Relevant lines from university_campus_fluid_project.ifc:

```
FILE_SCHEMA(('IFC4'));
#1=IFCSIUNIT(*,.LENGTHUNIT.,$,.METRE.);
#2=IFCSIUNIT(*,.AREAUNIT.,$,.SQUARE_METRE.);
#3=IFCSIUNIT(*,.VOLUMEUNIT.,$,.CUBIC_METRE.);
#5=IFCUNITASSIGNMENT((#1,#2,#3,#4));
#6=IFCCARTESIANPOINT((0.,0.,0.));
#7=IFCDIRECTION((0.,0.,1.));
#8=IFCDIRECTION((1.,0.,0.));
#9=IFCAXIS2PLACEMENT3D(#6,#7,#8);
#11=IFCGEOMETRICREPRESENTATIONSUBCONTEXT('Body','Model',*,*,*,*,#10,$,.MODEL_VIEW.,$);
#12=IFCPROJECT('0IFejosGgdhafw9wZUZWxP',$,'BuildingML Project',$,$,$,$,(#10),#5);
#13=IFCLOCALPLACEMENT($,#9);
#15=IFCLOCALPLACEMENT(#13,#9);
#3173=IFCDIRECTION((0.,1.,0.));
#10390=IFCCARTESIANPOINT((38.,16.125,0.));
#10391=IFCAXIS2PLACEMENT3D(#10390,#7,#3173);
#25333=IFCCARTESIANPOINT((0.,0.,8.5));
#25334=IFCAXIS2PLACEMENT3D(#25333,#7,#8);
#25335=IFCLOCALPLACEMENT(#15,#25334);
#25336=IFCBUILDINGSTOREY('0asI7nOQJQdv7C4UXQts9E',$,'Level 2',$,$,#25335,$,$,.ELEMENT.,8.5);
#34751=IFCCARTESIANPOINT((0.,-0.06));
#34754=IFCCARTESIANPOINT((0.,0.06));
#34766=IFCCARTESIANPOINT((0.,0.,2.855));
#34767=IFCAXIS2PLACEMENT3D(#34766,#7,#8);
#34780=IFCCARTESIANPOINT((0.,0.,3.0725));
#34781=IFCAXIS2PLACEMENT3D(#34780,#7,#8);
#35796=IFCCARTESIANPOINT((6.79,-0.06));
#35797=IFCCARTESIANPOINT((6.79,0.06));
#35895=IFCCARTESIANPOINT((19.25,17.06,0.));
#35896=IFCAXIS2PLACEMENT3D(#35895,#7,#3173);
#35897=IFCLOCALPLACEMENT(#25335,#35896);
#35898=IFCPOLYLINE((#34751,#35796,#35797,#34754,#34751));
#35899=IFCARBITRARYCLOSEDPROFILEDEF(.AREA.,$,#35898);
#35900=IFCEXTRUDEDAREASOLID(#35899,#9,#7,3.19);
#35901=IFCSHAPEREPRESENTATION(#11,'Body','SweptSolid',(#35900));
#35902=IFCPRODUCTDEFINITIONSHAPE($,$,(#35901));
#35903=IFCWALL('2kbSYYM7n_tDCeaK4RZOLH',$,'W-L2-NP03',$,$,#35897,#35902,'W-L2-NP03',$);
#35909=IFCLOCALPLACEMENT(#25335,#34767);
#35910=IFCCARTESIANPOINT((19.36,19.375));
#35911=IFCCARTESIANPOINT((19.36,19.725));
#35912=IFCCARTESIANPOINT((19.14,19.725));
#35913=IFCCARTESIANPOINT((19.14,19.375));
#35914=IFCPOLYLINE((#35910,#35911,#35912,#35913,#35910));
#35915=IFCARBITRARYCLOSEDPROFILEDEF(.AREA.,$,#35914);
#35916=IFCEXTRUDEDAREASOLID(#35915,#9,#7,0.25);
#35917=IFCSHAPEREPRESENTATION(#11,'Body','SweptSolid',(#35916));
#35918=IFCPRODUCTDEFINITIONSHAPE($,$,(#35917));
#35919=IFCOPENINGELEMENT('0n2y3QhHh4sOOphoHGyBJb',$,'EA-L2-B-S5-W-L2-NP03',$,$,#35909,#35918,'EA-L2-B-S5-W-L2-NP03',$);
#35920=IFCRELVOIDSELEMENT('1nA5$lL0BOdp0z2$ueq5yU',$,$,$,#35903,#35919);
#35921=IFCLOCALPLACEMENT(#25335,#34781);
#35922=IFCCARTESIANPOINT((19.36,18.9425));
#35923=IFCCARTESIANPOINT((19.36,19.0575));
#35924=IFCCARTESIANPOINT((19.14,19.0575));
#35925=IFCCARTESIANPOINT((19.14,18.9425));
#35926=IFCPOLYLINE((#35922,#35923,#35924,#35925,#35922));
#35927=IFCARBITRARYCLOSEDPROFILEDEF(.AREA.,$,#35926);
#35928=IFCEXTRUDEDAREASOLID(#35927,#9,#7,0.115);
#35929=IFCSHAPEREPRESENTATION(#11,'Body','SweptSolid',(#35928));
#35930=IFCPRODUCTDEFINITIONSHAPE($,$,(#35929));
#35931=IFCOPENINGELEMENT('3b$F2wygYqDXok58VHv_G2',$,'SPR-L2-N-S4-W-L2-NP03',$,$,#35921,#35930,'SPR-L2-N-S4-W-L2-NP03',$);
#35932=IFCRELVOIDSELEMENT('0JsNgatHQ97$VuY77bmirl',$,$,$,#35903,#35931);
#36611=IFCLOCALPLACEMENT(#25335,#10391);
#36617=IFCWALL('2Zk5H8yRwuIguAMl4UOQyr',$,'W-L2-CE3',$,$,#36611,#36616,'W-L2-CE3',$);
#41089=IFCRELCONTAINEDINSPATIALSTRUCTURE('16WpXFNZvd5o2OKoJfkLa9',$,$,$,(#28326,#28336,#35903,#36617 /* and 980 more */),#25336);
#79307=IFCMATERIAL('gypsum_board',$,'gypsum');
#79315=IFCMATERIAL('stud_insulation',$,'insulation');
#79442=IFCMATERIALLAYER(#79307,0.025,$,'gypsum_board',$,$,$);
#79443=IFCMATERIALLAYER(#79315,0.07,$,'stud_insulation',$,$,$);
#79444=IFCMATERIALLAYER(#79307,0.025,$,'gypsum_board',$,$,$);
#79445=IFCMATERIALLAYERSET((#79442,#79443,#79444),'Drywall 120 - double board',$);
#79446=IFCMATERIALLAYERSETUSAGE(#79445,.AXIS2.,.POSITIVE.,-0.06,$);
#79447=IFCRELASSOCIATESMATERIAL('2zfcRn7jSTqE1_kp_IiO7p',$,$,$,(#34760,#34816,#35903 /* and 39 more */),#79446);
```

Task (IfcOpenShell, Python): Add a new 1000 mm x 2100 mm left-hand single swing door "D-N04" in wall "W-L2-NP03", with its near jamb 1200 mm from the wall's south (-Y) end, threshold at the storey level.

```python
import numpy as np
import ifcopenshell
import ifcopenshell.api.feature
import ifcopenshell.api.geometry
import ifcopenshell.api.root
import ifcopenshell.api.spatial
import ifcopenshell.geom
import ifcopenshell.util.element
import ifcopenshell.util.placement
import ifcopenshell.util.representation
import ifcopenshell.util.shape
import ifcopenshell.util.unit

model = ifcopenshell.open("university_campus_fluid_project.ifc")
unit_scale = ifcopenshell.util.unit.calculate_unit_scale(model)
settings = ifcopenshell.geom.settings()


def volume(element):
    """Net volume in cubic metres, openings subtracted."""
    shape = ifcopenshell.geom.create_shape(settings, element)
    return ifcopenshell.util.shape.get_volume(shape.geometry)


wall = model.by_id(35903)
storey = ifcopenshell.util.element.get_container(wall, ifc_class="IfcBuildingStorey")
context = ifcopenshell.util.representation.get_context(model, "Model", "Body", "MODEL_VIEW")
before = volume(wall)

width, height, from_end, sill = 1, 2.1, 1.2, 0.0  # metres

# The wall runs along its own X axis, and the end named is its -X end.
wall_shape = ifcopenshell.geom.create_shape(settings, wall)
x, y, z = ifcopenshell.util.shape.get_vertices(wall_shape.geometry).T
start = x.min() + from_end
face, thickness = float(y.min()), float(y.max() - y.min())
wall_matrix = ifcopenshell.util.placement.get_local_placement(wall.ObjectPlacement)
level = ifcopenshell.util.placement.get_local_placement(storey.ObjectPlacement)[2, 3]


def in_wall(x, y):
    """Placement at x, y metres in the wall's axes, at sill height."""
    matrix = wall_matrix.copy()
    matrix[:, 3] = wall_matrix @ np.array([x / unit_scale, y / unit_scale, 0.0, 1.0])
    matrix[2, 3] = level + sill / unit_scale
    return matrix


# Opening: a box that overshoots both wall faces by 50 mm.
opening = ifcopenshell.api.root.create_entity(model, ifc_class="IfcOpeningElement", predefined_type="OPENING")
box = ifcopenshell.api.geometry.add_wall_representation(
    model, context=context, length=width, height=height, thickness=thickness + 0.1
)
ifcopenshell.api.geometry.assign_representation(model, product=opening, representation=box)
ifcopenshell.api.geometry.edit_object_placement(model, product=opening, matrix=in_wall(start, face - 0.05), is_si=False)
ifcopenshell.api.feature.add_feature(model, feature=opening, element=wall)

door = ifcopenshell.api.root.create_entity(model, ifc_class="IfcDoor", name="D-N04", predefined_type="DOOR")
door.OverallWidth, door.OverallHeight = width / unit_scale, height / unit_scale
door.OperationType = "SINGLE_SWING_LEFT"
body = ifcopenshell.api.geometry.add_door_representation(
    model,
    context=context,
    overall_width=door.OverallWidth,
    overall_height=door.OverallHeight,
    operation_type="SINGLE_SWING_LEFT",
    lining_properties={"LiningDepth": thickness / unit_scale, "ThresholdDepth": thickness / unit_scale},
)
ifcopenshell.api.geometry.assign_representation(model, product=door, representation=body)
ifcopenshell.api.spatial.assign_container(model, products=[door], relating_structure=storey)
ifcopenshell.api.feature.add_filling(model, opening=opening, element=door)

# The lining spans the wall, so the door starts at the wall face.
ifcopenshell.api.geometry.edit_object_placement(model, product=door, matrix=in_wall(start, face), is_si=False)

after = volume(wall)

print(f"wall volume {before:.3f} -> {after:.3f} m3")

model.write("university_campus_fluid_project_rev.ifc")
```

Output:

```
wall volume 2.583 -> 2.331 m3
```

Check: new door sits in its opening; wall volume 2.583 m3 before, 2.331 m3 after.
